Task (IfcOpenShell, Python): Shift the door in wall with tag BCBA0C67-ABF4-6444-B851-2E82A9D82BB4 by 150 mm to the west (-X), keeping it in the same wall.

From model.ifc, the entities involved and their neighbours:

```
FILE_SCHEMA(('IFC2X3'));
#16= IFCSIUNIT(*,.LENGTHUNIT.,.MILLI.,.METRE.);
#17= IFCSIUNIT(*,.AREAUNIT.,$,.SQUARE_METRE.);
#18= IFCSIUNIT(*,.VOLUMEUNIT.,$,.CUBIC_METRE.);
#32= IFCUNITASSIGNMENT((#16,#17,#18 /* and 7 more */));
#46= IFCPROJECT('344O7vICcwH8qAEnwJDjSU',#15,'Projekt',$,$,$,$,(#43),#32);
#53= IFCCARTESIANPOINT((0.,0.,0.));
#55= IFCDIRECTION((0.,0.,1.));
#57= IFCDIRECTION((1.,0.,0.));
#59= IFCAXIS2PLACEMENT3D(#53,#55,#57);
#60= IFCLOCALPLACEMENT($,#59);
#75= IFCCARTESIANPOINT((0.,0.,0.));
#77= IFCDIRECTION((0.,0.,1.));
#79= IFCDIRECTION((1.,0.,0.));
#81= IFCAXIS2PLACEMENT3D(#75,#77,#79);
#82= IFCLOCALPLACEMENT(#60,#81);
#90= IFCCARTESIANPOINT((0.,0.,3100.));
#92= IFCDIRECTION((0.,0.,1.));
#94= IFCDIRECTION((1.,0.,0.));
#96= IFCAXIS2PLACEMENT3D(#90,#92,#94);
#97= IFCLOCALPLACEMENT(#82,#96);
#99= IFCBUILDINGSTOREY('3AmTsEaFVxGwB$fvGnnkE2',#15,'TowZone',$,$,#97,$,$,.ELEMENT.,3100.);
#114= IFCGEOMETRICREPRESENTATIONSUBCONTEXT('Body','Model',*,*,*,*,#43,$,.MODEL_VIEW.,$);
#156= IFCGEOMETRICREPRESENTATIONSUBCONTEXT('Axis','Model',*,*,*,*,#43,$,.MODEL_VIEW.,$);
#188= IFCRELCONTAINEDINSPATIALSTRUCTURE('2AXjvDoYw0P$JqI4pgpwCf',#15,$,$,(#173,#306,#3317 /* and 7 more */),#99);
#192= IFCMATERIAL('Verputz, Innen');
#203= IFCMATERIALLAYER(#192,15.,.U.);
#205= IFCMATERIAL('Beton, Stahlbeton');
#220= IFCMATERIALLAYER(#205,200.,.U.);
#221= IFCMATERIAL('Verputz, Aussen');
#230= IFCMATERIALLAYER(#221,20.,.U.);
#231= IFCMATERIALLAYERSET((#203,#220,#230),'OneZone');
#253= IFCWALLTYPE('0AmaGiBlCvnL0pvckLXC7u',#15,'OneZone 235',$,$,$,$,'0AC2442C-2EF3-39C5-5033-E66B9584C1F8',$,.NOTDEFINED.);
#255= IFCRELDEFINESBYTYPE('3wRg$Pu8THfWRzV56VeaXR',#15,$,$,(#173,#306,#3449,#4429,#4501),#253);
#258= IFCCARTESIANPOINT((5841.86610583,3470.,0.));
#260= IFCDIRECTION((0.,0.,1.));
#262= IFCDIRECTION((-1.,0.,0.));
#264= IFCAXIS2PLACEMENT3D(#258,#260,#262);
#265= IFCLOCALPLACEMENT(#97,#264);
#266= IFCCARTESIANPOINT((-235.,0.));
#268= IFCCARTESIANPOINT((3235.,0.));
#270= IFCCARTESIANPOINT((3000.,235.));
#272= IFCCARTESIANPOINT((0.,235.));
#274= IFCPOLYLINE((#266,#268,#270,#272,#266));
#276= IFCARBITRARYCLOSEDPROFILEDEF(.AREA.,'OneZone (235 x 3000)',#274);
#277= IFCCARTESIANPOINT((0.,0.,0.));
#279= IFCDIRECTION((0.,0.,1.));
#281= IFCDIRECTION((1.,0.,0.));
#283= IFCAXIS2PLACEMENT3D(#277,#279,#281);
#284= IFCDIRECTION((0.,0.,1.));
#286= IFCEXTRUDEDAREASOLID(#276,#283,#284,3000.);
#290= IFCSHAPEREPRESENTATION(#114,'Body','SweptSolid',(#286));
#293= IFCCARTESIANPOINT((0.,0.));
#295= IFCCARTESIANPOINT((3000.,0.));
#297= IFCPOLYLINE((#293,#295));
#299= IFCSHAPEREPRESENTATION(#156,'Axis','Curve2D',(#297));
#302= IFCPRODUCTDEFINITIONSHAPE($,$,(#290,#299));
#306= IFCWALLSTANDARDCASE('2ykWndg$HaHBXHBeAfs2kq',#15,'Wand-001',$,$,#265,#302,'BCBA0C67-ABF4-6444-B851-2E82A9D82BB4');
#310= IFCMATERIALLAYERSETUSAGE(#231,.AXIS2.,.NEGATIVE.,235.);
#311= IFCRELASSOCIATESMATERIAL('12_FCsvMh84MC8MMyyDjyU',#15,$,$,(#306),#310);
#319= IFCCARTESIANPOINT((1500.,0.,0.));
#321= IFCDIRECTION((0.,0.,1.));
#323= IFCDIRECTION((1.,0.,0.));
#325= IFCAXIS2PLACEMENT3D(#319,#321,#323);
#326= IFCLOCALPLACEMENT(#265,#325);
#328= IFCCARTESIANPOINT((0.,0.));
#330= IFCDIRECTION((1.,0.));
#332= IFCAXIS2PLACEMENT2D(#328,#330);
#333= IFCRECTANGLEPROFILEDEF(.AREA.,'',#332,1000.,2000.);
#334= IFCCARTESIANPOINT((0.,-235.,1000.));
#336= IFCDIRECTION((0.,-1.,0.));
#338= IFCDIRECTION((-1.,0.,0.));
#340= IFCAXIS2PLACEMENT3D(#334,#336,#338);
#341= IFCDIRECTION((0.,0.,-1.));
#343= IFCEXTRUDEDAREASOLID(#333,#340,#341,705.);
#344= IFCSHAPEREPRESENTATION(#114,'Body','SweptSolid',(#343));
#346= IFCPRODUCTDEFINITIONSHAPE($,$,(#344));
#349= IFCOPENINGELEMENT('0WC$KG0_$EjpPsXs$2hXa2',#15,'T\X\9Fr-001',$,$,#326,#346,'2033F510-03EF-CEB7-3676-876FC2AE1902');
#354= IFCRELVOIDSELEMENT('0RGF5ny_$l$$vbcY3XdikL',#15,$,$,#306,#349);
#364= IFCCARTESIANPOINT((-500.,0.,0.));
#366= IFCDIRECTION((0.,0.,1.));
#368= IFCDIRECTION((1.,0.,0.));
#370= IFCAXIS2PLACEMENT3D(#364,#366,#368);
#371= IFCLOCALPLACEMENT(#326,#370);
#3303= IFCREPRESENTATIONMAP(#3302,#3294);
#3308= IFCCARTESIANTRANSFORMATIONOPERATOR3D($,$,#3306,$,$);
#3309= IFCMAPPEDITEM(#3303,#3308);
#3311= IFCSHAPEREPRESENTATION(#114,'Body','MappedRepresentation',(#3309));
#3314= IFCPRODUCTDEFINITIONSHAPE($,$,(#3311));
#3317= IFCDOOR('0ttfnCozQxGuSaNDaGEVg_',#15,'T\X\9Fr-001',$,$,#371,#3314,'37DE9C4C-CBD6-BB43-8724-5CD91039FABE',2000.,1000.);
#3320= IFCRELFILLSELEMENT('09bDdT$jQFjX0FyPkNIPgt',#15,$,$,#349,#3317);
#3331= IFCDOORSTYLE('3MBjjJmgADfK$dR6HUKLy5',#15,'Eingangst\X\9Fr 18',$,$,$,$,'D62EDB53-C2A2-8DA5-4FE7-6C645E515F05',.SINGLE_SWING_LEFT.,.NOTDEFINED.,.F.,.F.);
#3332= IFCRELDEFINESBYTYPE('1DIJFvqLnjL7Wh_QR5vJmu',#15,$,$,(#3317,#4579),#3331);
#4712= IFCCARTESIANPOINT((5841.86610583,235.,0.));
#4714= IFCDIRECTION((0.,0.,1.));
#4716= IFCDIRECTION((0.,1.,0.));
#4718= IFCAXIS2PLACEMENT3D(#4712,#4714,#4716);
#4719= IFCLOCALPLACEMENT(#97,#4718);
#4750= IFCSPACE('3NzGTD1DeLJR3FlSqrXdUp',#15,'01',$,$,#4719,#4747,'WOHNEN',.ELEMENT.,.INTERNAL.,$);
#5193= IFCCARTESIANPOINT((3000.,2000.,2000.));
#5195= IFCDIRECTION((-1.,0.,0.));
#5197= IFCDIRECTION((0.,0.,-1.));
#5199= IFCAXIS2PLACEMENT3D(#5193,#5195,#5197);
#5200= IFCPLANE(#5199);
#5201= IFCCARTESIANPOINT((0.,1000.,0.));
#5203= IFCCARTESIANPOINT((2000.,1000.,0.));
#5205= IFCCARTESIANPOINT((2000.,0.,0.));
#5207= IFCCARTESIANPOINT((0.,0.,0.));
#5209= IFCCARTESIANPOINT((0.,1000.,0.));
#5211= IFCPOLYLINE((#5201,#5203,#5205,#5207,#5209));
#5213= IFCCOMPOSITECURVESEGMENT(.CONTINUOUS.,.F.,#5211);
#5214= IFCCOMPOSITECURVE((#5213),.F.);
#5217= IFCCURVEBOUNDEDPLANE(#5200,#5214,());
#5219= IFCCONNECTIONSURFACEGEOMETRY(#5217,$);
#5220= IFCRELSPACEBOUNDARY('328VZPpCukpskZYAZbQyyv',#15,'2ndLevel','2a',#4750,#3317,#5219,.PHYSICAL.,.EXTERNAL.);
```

```python
import numpy as np
import ifcopenshell
import ifcopenshell.api.geometry
import ifcopenshell.util.placement

model = ifcopenshell.open("model.ifc")

door = model.by_id(3317)
opening = door.FillsVoids[0].RelatingOpeningElement
wall = opening.VoidsElements[0].RelatingBuildingElement

wall_matrix = ifcopenshell.util.placement.get_local_placement(wall.ObjectPlacement)
shift = wall_matrix[:3, 0] * 150.0
before = ifcopenshell.util.placement.get_local_placement(door.ObjectPlacement)[:3, 3].copy()

# The door is placed relative to its opening, so it follows when the opening moves.
matrix = ifcopenshell.util.placement.get_local_placement(opening.ObjectPlacement)
matrix[:3, 3] += shift
ifcopenshell.api.geometry.edit_object_placement(
    model, product=opening, matrix=matrix, is_si=False, should_transform_children=True
)

# Space boundary surfaces are stored in each space's coordinates; move them too.
for rel in door.ProvidesBoundaries:
    if not rel.ConnectionGeometry:
        continue
    surface = rel.ConnectionGeometry.SurfaceOnRelatingElement.BasisSurface
    space_matrix = ifcopenshell.util.placement.get_local_placement(rel.RelatingSpace.ObjectPlacement)
    point = np.array(surface.Position.Location.Coordinates) + space_matrix[:3, :3].T @ shift
    surface.Position = model.createIfcAxis2Placement3D(
        model.createIfcCartesianPoint(point.tolist()), surface.Position.Axis, surface.Position.RefDirection
    )

after = ifcopenshell.util.placement.get_local_placement(door.ObjectPlacement)[:3, 3]
print("door moved by", (after - before).round(3) + 0.0)

model.write("model_rev.ifc")
```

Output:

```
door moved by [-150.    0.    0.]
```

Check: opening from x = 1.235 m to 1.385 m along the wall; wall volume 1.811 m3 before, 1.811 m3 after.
